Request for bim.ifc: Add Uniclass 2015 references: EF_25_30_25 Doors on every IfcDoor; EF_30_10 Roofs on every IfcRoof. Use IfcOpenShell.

First a look at what the model holds.

```python
import ifcopenshell

model = ifcopenshell.open("bim.ifc")
print(model.schema)
print("classifications:", [c.Name for c in model.by_type("IfcClassification")])
for ifc_class in ("IfcDoor", "IfcRoof", "IfcStair", "IfcWall", "IfcWindow"):
    print(ifc_class, len(model.by_type(ifc_class)))
```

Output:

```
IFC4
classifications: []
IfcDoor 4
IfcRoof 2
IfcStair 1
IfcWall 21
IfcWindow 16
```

```python
import ifcopenshell
import ifcopenshell.api.classification

model = ifcopenshell.open("bim.ifc")

system = ifcopenshell.api.classification.add_classification(model, classification="Uniclass 2015")

codes = {
    "IfcDoor": ("EF_25_30_25", "Doors"),
    "IfcRoof": ("EF_30_10", "Roofs"),
}
for ifc_class, (code, name) in codes.items():
    products = model.by_type(ifc_class)
    ifcopenshell.api.classification.add_reference(
        model, products=products, classification=system, identification=code, name=name
    )
    print(code, len(products))

model.write("bim_updated.ifc")
```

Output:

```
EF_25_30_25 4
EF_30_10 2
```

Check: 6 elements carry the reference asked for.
